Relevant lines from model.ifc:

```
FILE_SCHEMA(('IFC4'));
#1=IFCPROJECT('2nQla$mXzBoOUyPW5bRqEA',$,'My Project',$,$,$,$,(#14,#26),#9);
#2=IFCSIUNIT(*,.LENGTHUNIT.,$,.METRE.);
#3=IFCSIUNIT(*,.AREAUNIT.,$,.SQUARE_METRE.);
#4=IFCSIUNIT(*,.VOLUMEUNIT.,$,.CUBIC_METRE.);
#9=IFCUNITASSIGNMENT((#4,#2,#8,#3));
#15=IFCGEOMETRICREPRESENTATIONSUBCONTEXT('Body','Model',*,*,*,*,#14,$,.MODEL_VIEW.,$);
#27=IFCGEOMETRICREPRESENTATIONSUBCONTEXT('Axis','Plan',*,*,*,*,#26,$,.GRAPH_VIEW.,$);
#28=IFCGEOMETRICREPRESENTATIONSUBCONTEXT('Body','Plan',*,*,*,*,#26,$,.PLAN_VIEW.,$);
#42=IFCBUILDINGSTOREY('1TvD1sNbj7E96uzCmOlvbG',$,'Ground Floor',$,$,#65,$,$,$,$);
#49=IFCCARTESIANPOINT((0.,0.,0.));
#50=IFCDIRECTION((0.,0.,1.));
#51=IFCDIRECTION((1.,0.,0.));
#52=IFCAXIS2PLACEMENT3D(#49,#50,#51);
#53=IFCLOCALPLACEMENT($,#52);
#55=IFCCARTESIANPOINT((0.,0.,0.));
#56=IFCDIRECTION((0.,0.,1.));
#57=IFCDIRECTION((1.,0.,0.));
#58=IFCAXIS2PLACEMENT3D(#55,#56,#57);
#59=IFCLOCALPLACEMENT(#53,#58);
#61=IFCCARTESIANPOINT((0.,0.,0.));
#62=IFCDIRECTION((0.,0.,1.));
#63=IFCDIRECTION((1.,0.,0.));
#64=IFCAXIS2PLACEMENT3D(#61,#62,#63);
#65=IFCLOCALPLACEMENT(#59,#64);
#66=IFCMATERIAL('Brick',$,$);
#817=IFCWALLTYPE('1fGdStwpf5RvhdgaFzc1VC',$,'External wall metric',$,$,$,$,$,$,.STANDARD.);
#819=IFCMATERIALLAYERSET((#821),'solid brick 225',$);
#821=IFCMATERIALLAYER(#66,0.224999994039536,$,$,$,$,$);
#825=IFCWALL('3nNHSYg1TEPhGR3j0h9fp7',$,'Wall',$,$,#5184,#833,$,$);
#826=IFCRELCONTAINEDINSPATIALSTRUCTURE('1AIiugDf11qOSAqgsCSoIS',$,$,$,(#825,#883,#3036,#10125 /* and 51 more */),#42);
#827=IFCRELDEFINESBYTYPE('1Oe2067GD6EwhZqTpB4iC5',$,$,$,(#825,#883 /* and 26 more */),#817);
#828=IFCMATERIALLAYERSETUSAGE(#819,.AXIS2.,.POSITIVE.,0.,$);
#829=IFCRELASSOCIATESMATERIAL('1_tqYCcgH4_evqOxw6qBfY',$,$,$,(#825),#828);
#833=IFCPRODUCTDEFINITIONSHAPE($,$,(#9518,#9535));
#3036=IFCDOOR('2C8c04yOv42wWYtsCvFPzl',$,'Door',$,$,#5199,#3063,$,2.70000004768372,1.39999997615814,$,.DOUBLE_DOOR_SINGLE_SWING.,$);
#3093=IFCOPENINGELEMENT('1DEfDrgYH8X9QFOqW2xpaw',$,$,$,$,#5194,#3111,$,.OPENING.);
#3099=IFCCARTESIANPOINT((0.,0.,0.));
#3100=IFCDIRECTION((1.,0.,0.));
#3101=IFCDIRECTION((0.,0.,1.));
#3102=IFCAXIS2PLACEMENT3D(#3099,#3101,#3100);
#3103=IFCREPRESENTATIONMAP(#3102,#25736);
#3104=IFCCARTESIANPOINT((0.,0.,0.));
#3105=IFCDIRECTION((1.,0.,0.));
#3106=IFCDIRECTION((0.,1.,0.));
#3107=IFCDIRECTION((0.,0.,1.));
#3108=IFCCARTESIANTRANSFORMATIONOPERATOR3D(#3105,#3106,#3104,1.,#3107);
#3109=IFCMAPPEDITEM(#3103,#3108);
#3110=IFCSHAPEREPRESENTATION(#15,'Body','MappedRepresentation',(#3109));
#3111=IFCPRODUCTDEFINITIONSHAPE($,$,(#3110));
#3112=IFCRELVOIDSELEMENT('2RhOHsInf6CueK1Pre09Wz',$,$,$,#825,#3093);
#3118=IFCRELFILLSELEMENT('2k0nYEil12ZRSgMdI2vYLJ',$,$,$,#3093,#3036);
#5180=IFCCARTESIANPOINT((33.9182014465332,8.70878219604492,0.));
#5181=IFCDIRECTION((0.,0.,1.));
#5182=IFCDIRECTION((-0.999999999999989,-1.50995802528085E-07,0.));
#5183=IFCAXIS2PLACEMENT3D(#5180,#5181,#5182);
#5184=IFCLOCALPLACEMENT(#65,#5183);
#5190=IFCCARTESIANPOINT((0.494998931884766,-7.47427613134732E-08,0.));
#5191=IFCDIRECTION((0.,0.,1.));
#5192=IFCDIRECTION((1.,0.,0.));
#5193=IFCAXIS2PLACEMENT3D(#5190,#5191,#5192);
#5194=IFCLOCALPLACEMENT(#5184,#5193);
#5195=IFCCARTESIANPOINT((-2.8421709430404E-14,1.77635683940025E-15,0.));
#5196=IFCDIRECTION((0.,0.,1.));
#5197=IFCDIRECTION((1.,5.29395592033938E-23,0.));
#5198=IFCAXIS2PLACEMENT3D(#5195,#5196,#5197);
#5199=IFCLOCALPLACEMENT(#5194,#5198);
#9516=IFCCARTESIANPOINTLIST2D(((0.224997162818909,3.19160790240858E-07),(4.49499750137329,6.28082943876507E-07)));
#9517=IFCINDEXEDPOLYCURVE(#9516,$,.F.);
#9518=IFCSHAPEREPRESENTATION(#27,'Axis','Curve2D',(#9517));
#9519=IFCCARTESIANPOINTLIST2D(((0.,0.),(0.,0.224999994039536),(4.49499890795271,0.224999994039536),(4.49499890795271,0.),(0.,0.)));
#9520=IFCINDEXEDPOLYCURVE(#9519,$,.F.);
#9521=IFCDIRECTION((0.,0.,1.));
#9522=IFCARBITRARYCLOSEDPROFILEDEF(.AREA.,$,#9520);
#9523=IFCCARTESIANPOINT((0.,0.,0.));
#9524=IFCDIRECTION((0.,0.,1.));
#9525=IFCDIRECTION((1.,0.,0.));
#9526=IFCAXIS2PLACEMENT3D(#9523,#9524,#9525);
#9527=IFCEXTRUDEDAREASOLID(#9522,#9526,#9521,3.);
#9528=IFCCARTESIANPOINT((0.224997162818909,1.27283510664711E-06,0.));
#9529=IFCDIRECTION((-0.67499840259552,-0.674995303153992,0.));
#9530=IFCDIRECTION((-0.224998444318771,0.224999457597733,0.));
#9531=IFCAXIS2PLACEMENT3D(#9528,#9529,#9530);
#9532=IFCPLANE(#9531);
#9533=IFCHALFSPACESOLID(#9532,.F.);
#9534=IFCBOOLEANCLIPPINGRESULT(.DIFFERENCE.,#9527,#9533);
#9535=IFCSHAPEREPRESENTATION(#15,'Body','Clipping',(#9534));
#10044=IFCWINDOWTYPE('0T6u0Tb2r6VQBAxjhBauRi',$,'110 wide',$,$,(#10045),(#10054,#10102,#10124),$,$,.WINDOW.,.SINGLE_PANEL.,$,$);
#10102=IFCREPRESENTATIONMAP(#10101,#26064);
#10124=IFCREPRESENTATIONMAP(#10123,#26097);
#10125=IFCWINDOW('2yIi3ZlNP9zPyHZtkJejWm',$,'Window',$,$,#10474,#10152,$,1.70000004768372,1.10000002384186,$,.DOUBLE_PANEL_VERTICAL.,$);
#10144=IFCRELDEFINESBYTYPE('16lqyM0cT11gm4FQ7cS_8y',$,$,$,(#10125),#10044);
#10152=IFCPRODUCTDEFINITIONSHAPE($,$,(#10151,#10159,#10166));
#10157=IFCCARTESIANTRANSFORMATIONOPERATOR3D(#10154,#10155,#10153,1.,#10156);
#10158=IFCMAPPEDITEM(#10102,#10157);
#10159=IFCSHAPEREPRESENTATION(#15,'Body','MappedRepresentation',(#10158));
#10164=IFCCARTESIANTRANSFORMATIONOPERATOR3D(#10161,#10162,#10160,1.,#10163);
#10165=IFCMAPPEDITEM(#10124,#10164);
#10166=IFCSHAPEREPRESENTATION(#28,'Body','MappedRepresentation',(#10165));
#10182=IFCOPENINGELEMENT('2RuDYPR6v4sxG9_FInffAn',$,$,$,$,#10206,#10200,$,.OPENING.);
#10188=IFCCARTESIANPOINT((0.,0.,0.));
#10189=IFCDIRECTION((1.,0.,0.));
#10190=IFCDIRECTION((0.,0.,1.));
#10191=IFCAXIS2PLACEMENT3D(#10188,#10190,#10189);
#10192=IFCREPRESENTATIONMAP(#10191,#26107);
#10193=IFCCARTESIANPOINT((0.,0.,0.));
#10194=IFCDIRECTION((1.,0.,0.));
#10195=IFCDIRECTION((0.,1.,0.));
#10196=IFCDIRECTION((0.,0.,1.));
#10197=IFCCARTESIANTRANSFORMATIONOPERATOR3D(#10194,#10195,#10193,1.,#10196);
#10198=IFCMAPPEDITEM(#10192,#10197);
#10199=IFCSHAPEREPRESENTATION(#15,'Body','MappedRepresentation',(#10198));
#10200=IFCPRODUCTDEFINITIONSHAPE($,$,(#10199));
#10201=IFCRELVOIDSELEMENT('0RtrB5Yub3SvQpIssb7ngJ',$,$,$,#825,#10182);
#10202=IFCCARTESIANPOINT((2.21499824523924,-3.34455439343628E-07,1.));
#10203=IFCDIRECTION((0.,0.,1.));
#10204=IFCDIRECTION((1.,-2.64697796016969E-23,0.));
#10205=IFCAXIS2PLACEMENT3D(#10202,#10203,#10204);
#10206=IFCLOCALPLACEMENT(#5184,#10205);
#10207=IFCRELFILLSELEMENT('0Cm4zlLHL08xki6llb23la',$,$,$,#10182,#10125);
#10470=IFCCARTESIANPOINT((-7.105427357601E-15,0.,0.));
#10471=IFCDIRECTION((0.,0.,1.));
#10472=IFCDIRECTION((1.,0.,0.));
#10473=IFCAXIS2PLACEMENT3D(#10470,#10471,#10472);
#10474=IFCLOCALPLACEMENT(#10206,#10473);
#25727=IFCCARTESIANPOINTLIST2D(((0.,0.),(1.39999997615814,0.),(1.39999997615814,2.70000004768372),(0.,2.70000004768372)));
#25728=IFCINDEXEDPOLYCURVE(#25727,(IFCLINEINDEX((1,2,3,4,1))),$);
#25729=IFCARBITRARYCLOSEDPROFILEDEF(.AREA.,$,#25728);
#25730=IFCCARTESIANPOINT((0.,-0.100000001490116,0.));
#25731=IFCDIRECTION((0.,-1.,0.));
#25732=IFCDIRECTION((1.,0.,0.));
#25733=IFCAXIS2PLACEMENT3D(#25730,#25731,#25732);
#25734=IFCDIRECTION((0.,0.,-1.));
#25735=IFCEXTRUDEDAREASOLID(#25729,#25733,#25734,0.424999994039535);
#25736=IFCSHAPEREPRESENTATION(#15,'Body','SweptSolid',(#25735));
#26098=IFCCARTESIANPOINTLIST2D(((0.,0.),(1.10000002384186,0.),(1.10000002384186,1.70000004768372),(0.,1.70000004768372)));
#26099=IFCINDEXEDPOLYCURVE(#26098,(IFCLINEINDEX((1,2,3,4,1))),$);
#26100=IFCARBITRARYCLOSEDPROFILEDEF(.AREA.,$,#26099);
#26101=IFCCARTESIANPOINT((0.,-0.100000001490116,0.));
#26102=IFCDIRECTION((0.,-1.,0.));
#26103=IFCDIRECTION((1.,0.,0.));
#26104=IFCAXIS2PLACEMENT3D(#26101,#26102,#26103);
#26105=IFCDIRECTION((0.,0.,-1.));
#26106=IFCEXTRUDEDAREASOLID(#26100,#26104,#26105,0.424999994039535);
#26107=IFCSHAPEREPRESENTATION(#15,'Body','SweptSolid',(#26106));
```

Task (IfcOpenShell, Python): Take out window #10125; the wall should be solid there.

```python
import ifcopenshell
import ifcopenshell.api.feature
import ifcopenshell.api.root
import ifcopenshell.geom
import ifcopenshell.util.shape

model = ifcopenshell.open("model.ifc")
settings = ifcopenshell.geom.settings()


def volume(element):
    """Net volume in cubic metres, openings subtracted."""
    shape = ifcopenshell.geom.create_shape(settings, element)
    return ifcopenshell.util.shape.get_volume(shape.geometry)


window = model.by_guid("2yIi3ZlNP9zPyHZtkJejWm")
opening = window.FillsVoids[0].RelatingOpeningElement
wall = opening.VoidsElements[0].RelatingBuildingElement
before = volume(wall)

ifcopenshell.api.root.remove_product(model, product=window)
ifcopenshell.api.feature.remove_feature(model, feature=opening)

after = volume(wall)

print(f"wall volume {before:.3f} -> {after:.3f} m3")

model.write("model_v2.ifc")
```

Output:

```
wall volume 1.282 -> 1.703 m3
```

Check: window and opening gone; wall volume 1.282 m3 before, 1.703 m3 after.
